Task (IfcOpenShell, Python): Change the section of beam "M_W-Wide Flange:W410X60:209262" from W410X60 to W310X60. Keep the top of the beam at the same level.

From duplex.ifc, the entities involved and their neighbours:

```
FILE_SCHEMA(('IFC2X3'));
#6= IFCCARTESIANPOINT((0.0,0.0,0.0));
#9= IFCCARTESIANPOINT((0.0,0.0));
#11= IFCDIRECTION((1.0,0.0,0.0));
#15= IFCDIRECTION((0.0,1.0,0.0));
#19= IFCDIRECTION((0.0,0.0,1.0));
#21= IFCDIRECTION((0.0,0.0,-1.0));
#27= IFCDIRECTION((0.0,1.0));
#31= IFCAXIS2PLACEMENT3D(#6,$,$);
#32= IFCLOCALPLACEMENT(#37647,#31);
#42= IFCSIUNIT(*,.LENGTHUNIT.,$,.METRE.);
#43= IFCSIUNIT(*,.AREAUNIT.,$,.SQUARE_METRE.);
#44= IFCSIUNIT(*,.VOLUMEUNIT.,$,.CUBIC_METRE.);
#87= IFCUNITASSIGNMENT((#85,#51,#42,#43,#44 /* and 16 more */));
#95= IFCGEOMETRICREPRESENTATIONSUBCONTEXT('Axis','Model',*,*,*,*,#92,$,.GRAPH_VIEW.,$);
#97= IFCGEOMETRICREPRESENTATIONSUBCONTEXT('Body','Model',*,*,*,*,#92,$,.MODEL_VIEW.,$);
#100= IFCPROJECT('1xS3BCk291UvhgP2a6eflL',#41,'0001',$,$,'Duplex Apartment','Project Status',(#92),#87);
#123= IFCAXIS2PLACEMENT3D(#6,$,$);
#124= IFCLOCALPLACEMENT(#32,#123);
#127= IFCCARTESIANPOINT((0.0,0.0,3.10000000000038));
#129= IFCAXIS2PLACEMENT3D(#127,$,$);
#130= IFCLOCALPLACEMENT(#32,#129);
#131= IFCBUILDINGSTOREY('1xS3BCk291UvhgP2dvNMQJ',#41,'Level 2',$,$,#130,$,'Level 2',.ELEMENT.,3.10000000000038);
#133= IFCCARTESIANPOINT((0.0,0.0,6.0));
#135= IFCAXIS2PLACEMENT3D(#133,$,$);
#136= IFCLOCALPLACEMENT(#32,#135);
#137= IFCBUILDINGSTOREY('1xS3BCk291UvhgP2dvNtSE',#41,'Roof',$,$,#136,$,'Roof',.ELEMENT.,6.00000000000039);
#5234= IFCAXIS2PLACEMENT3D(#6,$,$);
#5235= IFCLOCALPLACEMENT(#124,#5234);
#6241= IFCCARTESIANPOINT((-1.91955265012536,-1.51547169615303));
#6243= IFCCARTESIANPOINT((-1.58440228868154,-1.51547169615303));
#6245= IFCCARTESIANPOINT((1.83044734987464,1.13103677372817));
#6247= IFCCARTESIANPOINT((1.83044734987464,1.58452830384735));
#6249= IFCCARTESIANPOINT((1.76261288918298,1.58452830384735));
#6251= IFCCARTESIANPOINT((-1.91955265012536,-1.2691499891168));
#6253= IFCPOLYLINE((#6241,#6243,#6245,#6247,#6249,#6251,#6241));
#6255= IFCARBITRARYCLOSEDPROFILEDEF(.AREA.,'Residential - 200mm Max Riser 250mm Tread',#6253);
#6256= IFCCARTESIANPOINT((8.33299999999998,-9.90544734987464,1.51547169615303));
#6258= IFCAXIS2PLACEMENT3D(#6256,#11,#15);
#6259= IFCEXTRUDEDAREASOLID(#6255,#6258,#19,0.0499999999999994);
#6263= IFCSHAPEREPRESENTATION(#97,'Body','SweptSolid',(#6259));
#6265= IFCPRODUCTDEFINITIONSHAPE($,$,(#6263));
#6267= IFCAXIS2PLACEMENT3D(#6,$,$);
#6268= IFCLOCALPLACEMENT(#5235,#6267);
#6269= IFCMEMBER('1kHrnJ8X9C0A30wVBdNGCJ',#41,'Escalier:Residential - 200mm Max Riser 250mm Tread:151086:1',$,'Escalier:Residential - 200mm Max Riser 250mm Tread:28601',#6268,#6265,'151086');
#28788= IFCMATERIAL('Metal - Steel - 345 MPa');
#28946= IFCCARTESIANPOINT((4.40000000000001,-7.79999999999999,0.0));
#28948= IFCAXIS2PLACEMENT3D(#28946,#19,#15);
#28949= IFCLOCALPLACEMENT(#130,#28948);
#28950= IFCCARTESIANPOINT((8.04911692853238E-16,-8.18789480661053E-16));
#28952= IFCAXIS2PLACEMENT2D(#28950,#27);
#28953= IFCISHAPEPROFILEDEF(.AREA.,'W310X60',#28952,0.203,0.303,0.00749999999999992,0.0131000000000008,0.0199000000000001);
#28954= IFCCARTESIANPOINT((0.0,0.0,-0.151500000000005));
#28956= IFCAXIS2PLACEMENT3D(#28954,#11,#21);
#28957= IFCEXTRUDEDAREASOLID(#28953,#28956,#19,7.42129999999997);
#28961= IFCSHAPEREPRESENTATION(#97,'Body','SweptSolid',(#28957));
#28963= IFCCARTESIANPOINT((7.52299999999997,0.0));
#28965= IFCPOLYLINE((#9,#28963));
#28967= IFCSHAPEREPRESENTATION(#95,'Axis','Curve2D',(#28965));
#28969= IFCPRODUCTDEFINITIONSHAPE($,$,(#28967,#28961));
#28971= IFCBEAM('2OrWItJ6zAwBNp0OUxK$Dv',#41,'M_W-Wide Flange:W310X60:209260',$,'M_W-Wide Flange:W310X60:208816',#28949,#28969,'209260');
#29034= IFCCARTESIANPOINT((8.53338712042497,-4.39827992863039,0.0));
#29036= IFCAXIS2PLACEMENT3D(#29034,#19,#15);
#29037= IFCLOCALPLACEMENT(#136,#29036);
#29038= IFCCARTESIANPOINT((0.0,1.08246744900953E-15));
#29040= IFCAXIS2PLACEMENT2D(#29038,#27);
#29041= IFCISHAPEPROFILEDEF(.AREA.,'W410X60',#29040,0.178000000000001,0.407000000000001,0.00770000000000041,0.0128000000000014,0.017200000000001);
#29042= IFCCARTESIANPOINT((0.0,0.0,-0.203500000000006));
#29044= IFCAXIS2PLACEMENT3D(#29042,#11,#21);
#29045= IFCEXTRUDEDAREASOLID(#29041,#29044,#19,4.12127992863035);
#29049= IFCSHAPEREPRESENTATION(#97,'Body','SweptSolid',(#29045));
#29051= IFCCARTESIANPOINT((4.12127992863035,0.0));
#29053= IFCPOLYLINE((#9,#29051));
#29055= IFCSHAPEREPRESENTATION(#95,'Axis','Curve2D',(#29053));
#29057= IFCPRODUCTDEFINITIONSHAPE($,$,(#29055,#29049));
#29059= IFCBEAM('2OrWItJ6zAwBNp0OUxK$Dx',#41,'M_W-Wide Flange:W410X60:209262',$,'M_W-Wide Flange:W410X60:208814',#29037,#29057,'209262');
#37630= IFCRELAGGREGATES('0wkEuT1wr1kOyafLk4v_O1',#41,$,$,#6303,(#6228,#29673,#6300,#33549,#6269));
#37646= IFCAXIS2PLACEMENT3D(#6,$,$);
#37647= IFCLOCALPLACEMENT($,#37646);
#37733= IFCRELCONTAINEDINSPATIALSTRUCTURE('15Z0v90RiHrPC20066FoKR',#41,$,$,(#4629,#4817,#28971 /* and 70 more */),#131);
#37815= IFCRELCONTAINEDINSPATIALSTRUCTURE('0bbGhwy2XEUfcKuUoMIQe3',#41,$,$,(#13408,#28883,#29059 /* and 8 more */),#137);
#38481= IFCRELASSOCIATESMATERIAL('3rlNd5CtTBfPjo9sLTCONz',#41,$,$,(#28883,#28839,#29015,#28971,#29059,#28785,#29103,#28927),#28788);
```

```python
import ifcopenshell
import ifcopenshell.util.element
import ifcopenshell.util.representation

model = ifcopenshell.open("duplex.ifc")

member = model.by_id(29059)
source = next(p for p in model.by_type("IfcIShapeProfileDef") if p.ProfileName == "W310X60")

body = ifcopenshell.util.representation.get_representation(member, "Model", "Body")
solid = body.Items[0]
old_profile = solid.SweptArea

# Copy the section's sizes but keep this member's own profile position.
profile = ifcopenshell.util.element.copy(model, source)
# Profiles are centred, so shift by half the change in depth to hold the top.
shift = (old_profile.OverallDepth - profile.OverallDepth) / 2
x, y = old_profile.Position.Location.Coordinates
up = (-1.0, 0.0)  # upwards, in the solid's own plane
location = model.createIfcCartesianPoint((x + up[0] * shift, y + up[1] * shift))
profile.Position = model.createIfcAxis2Placement2D(location, old_profile.Position.RefDirection)
solid.SweptArea = profile
if not model.get_total_inverses(old_profile):
    ifcopenshell.util.element.remove_deep2(model, old_profile)
member.Name = member.Name.replace("W410X60", "W310X60")
member.ObjectType = member.ObjectType.replace("W410X60", "W310X60")

print(solid.SweptArea)

model.write("duplex_edited.ifc")
```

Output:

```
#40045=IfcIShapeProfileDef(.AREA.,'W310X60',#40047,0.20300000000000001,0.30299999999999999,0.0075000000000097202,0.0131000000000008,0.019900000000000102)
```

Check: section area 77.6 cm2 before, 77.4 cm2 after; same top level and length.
